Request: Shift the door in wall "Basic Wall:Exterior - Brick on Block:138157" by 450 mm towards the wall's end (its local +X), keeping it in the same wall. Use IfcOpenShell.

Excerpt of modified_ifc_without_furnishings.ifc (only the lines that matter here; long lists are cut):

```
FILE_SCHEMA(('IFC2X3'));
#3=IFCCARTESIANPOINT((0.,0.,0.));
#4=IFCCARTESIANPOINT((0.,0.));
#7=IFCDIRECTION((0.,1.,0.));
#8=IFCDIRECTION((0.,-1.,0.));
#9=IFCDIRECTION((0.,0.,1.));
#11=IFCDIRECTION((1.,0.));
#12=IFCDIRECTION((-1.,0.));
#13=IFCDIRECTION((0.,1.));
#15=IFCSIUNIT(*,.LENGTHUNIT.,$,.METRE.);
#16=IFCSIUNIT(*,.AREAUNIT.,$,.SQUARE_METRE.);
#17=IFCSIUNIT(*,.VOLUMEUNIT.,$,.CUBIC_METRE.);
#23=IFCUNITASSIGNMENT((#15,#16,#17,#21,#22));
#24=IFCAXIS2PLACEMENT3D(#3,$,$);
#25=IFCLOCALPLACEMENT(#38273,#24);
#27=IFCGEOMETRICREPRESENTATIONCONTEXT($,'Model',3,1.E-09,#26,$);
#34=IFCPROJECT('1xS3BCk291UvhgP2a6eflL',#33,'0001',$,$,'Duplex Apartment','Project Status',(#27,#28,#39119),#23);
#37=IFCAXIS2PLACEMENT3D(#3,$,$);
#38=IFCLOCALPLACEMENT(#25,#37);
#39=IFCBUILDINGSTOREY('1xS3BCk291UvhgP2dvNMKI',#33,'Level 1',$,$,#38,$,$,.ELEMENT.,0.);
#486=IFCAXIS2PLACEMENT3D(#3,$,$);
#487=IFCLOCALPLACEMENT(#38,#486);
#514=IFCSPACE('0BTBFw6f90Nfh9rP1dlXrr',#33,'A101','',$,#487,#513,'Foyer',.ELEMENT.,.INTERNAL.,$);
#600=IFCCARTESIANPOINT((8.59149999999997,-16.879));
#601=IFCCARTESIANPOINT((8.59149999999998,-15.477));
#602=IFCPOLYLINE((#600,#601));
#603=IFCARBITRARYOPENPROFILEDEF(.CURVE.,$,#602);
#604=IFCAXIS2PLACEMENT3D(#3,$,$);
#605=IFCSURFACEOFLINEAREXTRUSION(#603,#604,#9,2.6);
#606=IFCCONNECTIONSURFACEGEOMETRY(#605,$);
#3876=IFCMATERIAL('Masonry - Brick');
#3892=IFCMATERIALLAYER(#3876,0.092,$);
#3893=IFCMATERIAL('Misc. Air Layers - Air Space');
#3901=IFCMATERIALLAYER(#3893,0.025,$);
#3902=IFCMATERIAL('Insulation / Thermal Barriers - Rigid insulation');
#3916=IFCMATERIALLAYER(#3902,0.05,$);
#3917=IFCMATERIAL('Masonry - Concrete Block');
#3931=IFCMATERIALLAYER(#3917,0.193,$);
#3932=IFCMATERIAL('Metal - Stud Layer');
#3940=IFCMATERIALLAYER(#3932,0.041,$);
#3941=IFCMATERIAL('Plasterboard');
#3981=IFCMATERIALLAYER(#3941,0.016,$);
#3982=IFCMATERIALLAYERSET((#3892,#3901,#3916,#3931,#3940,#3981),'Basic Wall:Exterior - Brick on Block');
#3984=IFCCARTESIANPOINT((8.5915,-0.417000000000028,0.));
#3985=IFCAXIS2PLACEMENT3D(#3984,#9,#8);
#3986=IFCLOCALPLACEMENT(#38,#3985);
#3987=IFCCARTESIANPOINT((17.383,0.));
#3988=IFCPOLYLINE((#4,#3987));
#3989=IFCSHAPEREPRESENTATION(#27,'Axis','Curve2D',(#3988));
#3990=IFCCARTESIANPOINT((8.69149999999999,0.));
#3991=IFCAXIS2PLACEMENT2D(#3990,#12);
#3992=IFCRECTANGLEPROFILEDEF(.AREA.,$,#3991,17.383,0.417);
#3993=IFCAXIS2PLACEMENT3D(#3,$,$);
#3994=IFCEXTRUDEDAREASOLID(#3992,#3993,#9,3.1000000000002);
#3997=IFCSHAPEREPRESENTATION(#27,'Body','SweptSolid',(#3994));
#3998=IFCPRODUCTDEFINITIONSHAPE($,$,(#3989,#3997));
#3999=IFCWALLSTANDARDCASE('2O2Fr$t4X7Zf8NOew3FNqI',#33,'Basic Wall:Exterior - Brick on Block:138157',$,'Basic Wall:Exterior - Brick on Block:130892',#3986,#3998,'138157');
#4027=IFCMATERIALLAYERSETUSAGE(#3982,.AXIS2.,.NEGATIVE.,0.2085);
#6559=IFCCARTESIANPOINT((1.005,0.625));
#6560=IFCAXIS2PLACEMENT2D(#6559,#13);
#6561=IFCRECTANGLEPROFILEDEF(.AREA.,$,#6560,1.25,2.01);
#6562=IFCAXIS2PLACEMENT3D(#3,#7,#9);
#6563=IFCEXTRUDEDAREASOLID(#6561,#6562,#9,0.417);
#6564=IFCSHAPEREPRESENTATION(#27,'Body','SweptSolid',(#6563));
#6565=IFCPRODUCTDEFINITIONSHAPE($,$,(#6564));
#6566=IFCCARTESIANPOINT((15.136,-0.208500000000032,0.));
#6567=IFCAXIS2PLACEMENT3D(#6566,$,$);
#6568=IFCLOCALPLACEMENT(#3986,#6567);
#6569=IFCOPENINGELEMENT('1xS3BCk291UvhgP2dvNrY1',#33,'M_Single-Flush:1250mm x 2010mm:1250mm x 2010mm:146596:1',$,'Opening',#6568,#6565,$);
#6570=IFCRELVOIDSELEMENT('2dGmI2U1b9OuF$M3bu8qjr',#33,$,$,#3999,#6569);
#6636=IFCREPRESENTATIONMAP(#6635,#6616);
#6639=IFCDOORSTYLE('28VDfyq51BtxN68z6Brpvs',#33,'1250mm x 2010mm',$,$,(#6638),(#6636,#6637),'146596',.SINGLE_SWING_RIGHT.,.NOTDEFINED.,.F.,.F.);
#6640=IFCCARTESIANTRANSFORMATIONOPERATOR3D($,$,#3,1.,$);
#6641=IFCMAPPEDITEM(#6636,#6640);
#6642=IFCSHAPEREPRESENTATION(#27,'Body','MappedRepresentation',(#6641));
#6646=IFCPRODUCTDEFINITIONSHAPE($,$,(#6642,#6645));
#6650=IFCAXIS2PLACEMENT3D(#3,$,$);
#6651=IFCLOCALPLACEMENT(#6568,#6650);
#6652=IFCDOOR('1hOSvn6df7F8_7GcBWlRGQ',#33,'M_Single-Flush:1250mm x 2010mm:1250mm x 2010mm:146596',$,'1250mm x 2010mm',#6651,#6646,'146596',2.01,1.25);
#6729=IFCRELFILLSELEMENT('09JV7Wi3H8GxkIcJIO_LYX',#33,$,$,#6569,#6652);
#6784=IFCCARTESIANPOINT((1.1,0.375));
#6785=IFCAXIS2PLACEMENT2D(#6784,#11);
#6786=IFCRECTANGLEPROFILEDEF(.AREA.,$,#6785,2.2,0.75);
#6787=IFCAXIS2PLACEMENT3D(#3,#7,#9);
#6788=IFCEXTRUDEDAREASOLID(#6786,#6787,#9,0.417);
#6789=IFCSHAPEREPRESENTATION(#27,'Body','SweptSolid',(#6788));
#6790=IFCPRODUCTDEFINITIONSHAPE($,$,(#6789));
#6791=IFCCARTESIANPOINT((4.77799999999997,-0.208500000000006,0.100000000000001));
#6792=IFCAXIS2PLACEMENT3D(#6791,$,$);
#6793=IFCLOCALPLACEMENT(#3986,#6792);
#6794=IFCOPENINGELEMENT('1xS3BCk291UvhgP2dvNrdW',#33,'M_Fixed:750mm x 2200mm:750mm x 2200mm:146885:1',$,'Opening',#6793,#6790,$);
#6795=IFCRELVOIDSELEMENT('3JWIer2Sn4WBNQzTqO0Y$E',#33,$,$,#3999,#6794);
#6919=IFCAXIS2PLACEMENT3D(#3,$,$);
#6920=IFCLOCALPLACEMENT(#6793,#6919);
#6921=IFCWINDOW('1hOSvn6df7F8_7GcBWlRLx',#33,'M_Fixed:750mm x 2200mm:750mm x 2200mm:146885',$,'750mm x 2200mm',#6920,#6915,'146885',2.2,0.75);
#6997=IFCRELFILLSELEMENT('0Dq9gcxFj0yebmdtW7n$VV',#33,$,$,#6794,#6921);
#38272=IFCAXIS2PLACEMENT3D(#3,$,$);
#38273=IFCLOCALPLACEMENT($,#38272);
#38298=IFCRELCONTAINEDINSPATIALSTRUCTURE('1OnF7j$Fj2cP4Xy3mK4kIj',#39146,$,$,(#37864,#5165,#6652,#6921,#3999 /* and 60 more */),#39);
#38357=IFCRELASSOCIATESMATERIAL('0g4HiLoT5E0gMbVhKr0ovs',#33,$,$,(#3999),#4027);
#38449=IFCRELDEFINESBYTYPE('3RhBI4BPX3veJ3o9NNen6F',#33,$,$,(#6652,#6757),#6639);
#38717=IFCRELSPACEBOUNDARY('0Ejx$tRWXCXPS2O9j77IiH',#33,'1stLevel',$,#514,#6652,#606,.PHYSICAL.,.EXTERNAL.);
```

```python
import numpy as np
import ifcopenshell
import ifcopenshell.api.geometry
import ifcopenshell.util.placement
import ifcopenshell.util.unit

model = ifcopenshell.open("modified_ifc_without_furnishings.ifc")
unit_scale = ifcopenshell.util.unit.calculate_unit_scale(model)

door = model.by_guid("1hOSvn6df7F8_7GcBWlRGQ")
opening = door.FillsVoids[0].RelatingOpeningElement
wall = opening.VoidsElements[0].RelatingBuildingElement

wall_matrix = ifcopenshell.util.placement.get_local_placement(wall.ObjectPlacement)
shift = wall_matrix[:3, 0] * 0.45 / unit_scale
before = ifcopenshell.util.placement.get_local_placement(door.ObjectPlacement)[:3, 3].copy()

# The door is placed relative to its opening, so it follows when the opening moves.
matrix = ifcopenshell.util.placement.get_local_placement(opening.ObjectPlacement)
matrix[:3, 3] += shift
ifcopenshell.api.geometry.edit_object_placement(
    model, product=opening, matrix=matrix, is_si=False, should_transform_children=True
)

# Space boundary surfaces are stored in each space's coordinates; move them too.
for rel in door.ProvidesBoundaries:
    if not rel.ConnectionGeometry:
        continue
    surface = rel.ConnectionGeometry.SurfaceOnRelatingElement
    space_matrix = ifcopenshell.util.placement.get_local_placement(rel.RelatingSpace.ObjectPlacement)
    point = np.array(surface.Position.Location.Coordinates) + space_matrix[:3, :3].T @ shift
    surface.Position = model.createIfcAxis2Placement3D(
        model.createIfcCartesianPoint(point.tolist()), surface.Position.Axis, surface.Position.RefDirection
    )

after = ifcopenshell.util.placement.get_local_placement(door.ObjectPlacement)[:3, 3]
print("door moved by", (after - before).round(3) + 0.0)

model.write("modified_ifc_without_furnishings_v2.ifc")
```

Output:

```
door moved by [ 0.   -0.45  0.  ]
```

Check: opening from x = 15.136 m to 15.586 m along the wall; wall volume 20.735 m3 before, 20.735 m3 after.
